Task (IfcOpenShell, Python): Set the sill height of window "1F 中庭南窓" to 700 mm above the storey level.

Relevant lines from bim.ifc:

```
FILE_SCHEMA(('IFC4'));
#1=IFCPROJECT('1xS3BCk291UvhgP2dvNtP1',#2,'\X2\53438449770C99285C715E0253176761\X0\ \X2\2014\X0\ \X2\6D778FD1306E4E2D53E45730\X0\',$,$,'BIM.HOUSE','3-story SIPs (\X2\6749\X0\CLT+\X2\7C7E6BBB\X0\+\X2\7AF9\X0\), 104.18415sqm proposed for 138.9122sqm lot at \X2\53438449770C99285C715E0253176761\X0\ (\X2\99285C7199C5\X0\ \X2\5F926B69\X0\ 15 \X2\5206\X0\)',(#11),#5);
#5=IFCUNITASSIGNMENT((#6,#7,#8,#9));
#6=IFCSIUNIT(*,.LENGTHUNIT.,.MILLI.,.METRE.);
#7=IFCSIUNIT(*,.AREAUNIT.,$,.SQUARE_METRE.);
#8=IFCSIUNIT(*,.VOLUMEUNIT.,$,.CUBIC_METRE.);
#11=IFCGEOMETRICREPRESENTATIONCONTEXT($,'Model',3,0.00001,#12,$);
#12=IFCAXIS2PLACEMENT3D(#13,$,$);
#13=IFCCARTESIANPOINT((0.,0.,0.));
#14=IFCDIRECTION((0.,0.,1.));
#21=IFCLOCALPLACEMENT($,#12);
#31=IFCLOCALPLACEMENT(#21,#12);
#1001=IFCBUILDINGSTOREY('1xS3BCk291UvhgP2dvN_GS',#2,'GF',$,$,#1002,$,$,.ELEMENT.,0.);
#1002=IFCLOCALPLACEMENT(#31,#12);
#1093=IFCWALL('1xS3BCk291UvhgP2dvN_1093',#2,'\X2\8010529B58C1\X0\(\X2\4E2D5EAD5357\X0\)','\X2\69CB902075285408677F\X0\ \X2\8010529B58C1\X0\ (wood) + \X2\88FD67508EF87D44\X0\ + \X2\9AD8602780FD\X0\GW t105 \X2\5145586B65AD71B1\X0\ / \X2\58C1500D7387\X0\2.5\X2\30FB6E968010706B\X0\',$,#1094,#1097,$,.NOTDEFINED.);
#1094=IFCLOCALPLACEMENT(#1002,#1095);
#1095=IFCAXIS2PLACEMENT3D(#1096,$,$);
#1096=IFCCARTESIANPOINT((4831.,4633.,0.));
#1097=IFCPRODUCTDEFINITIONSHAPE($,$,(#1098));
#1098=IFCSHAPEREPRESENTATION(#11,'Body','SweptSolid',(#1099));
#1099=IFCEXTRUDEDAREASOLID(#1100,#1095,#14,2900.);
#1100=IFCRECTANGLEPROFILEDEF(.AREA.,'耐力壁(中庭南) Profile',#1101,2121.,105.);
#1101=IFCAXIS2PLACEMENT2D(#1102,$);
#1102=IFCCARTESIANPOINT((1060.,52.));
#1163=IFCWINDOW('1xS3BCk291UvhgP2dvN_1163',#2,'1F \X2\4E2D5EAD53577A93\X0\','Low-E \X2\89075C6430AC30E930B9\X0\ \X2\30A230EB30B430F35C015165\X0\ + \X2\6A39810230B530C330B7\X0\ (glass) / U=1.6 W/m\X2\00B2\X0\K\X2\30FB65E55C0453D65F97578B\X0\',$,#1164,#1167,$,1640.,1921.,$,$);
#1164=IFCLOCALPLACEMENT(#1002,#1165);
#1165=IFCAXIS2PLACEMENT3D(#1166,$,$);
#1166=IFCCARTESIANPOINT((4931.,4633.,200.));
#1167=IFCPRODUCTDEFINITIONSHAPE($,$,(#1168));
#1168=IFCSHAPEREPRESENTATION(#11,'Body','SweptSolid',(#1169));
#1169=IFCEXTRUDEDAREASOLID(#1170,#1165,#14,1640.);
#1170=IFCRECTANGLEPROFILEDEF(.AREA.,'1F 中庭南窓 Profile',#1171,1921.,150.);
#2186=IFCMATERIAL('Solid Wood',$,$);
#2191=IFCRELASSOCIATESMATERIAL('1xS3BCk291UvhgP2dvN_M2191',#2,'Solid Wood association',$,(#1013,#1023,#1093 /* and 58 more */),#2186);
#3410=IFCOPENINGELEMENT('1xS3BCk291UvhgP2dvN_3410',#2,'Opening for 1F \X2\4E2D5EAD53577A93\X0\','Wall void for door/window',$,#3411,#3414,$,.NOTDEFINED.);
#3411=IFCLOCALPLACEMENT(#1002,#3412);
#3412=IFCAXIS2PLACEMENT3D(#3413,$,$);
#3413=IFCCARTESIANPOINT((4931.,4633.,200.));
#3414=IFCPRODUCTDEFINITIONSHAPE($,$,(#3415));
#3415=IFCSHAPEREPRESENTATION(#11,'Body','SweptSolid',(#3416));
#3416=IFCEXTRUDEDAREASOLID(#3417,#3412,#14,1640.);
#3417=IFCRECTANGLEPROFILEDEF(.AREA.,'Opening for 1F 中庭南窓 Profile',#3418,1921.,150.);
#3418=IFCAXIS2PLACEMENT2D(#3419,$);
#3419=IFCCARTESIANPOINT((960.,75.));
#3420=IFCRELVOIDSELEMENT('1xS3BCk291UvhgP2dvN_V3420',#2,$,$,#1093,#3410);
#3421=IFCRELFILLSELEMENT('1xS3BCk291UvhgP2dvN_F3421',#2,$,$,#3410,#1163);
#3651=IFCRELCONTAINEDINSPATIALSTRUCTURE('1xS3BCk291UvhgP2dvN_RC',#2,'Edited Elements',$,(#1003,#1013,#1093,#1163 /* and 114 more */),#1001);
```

```python
import numpy as np
import ifcopenshell
import ifcopenshell.api.geometry
import ifcopenshell.geom
import ifcopenshell.util.element
import ifcopenshell.util.placement
import ifcopenshell.util.shape
import ifcopenshell.util.unit

model = ifcopenshell.open("bim.ifc")
unit_scale = ifcopenshell.util.unit.calculate_unit_scale(model)

window = model.by_id(1163)
opening = window.FillsVoids[0].RelatingOpeningElement
storey = ifcopenshell.util.element.get_container(window, ifc_class="IfcBuildingStorey")
level = ifcopenshell.util.placement.get_local_placement(storey.ObjectPlacement)[2, 3]

# The opening's origin need not be at the sill, so measure its lowest point.
shape = ifcopenshell.geom.create_shape(ifcopenshell.geom.settings(), opening)
bottom = ifcopenshell.util.shape.get_shape_bottom_elevation(shape, shape.geometry) / unit_scale
dz = level + 700.0 - bottom

shift = np.array([0.0, 0.0, dz])
# The window is not placed relative to its opening, so move both.
for product in (opening, window):
    matrix = ifcopenshell.util.placement.get_local_placement(product.ObjectPlacement)
    matrix[:3, 3] += shift
    ifcopenshell.api.geometry.edit_object_placement(model, product=product, matrix=matrix, is_si=False)

print(f"moved by {dz * unit_scale:+.3f} m")

model.write("bim_edited.ifc")
```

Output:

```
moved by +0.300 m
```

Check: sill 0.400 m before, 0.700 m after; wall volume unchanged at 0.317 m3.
